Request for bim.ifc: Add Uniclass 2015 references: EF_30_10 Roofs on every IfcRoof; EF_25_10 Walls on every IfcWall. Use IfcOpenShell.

First a look at what the model holds.

```python
import ifcopenshell

model = ifcopenshell.open("bim.ifc")
print(model.schema)
print("classifications:", [c.Name for c in model.by_type("IfcClassification")])
for ifc_class in ("IfcDoor", "IfcRoof", "IfcStair", "IfcWall", "IfcWindow"):
    print(ifc_class, len(model.by_type(ifc_class)))
```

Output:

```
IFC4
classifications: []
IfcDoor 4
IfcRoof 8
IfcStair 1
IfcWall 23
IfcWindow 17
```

```python
import ifcopenshell
import ifcopenshell.api.classification

model = ifcopenshell.open("bim.ifc")

system = ifcopenshell.api.classification.add_classification(model, classification="Uniclass 2015")

codes = {
    "IfcRoof": ("EF_30_10", "Roofs"),
    "IfcWall": ("EF_25_10", "Walls"),
}
for ifc_class, (code, name) in codes.items():
    products = model.by_type(ifc_class)
    ifcopenshell.api.classification.add_reference(
        model, products=products, classification=system, identification=code, name=name
    )
    print(code, len(products))

model.write("bim_updated.ifc")
```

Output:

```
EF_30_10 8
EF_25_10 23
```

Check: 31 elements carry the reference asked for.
